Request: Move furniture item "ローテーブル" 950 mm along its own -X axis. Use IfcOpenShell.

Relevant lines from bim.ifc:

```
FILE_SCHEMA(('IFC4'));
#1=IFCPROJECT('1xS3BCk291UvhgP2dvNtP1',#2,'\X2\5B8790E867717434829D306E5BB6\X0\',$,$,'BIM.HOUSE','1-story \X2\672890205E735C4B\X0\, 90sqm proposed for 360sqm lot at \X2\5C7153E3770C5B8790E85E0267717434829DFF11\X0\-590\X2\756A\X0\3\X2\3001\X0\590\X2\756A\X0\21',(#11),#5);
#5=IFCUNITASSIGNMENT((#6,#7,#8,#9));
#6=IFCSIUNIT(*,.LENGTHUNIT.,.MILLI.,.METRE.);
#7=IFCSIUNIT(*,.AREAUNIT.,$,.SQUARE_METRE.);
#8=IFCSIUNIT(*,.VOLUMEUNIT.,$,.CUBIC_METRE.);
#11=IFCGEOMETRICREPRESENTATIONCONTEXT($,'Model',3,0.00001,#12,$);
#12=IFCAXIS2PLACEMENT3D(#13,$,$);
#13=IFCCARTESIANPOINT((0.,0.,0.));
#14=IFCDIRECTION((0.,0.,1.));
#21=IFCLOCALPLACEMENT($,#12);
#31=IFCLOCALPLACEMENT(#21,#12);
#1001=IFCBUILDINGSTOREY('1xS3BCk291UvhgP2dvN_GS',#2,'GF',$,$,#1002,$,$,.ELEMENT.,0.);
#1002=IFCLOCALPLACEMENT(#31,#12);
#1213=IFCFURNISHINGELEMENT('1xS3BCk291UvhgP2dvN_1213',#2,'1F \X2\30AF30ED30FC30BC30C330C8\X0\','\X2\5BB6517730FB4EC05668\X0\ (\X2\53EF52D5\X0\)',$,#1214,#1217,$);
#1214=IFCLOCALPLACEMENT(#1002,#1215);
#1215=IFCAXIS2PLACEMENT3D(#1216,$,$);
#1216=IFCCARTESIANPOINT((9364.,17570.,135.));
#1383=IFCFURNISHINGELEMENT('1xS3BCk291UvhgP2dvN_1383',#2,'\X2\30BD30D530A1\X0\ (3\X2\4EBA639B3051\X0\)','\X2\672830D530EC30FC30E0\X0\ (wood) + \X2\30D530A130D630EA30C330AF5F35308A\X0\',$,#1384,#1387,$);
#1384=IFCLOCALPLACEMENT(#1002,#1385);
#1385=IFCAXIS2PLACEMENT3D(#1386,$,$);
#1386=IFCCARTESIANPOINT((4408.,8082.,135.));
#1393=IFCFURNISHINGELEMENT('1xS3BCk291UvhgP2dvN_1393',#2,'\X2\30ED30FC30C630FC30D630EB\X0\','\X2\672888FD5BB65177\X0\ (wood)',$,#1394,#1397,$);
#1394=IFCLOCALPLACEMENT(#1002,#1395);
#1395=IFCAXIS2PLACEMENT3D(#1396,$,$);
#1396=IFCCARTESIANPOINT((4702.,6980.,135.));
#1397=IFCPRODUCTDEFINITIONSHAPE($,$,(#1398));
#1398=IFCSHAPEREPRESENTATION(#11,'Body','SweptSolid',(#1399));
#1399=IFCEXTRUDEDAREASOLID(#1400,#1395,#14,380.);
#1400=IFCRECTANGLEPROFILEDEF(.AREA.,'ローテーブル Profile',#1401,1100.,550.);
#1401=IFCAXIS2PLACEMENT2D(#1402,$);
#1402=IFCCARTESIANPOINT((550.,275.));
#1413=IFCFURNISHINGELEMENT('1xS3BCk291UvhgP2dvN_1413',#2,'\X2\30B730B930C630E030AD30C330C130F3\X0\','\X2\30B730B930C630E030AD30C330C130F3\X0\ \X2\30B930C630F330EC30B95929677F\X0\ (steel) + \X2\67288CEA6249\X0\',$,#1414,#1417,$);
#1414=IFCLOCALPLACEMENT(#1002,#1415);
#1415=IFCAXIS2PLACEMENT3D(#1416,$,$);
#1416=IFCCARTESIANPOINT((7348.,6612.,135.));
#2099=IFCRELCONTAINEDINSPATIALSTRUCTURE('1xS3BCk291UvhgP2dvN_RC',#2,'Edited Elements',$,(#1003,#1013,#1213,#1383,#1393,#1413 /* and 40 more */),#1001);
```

```python
import ifcopenshell
import ifcopenshell.api.geometry
import ifcopenshell.util.placement
import ifcopenshell.util.unit

model = ifcopenshell.open("bim.ifc")
unit_scale = ifcopenshell.util.unit.calculate_unit_scale(model)

item = model.by_guid("1xS3BCk291UvhgP2dvN_1393")
matrix = ifcopenshell.util.placement.get_local_placement(item.ObjectPlacement)
matrix[:3, 3] -= matrix[:3, 0] * 0.95 / unit_scale
ifcopenshell.api.geometry.edit_object_placement(model, product=item, matrix=matrix, is_si=False)

print(ifcopenshell.util.placement.get_local_placement(item.ObjectPlacement).round(3) + 0.0)

model.write("bim_rev.ifc")
```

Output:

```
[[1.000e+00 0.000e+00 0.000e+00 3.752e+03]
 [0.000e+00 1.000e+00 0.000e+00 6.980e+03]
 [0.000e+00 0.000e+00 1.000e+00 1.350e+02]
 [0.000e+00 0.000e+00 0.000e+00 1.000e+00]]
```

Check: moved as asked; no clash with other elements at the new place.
